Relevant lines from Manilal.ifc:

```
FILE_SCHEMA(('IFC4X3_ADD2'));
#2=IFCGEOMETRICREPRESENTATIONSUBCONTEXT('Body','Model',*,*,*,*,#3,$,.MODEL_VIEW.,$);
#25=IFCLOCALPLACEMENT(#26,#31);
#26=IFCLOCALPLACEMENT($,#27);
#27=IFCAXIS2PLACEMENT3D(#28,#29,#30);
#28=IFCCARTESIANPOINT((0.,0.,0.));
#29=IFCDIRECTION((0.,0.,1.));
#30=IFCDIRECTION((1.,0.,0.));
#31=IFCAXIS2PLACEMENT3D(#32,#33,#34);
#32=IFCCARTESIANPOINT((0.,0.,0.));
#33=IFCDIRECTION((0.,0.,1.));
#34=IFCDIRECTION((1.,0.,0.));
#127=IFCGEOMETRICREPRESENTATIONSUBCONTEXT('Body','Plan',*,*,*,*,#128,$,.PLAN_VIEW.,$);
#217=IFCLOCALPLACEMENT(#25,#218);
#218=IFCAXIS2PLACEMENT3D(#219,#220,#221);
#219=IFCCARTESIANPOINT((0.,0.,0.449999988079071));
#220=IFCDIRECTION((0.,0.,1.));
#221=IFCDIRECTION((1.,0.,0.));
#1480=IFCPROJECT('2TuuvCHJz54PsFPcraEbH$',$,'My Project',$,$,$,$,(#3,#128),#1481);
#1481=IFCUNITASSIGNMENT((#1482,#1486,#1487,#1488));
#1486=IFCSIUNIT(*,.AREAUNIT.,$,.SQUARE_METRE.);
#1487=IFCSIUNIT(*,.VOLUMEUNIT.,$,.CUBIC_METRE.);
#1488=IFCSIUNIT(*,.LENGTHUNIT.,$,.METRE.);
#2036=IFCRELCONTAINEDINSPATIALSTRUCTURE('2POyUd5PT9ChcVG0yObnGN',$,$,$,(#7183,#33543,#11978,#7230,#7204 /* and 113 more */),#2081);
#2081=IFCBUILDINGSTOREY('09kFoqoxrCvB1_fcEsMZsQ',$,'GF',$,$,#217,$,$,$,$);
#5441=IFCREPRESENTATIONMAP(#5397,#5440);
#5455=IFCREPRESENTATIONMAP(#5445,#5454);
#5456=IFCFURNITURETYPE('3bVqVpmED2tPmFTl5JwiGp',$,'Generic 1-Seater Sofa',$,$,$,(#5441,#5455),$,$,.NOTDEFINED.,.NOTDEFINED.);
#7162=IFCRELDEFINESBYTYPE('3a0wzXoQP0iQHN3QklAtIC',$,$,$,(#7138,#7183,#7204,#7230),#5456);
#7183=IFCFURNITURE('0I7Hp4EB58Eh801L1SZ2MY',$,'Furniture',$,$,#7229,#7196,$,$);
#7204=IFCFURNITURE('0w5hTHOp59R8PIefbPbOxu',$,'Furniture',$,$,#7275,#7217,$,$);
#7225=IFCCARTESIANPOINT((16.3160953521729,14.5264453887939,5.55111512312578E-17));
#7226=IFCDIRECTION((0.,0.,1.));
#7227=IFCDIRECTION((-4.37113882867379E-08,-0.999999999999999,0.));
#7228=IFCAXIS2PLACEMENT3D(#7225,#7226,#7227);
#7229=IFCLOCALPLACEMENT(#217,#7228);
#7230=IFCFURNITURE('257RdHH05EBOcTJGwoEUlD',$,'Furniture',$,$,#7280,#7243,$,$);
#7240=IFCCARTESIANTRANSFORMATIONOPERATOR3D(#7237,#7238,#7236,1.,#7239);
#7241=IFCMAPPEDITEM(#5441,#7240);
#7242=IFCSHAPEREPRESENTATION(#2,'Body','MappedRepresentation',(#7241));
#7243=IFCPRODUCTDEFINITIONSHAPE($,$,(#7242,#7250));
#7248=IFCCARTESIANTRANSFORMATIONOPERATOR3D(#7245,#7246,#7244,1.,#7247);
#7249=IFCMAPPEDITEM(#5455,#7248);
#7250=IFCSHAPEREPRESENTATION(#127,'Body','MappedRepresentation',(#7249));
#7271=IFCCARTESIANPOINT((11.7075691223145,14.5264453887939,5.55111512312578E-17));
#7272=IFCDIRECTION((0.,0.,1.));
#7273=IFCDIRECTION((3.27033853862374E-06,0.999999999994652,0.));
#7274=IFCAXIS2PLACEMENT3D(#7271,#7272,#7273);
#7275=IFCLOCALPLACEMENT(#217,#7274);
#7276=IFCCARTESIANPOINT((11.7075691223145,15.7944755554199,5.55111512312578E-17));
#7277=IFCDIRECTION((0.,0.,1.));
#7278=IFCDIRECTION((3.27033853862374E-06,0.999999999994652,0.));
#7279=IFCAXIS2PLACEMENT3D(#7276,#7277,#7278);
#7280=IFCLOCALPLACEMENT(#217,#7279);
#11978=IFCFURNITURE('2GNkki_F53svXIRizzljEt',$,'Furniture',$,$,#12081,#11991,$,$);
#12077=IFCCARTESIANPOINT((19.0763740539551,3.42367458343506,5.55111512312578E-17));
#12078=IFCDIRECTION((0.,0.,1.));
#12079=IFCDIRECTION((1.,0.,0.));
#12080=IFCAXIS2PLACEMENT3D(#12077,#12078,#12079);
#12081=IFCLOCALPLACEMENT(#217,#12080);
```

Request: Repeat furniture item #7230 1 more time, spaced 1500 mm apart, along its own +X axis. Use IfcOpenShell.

```python
import ifcopenshell
import ifcopenshell.api.geometry
import ifcopenshell.api.root
import ifcopenshell.util.element
import ifcopenshell.util.placement

model = ifcopenshell.open("Manilal.ifc")

source = model.by_id(7230)
base = ifcopenshell.util.placement.get_local_placement(source.ObjectPlacement)
step = base[:3, 0] * 1.5

for i in range(1, 2):
    copy = ifcopenshell.api.root.copy_class(model, product=source)
    copy.Representation = ifcopenshell.util.element.copy_deep(
        model, source.Representation, exclude=["IfcGeometricRepresentationContext", "IfcRepresentationMap"]
    )
    matrix = base.copy()
    matrix[:3, 3] += i * step
    print("added at", matrix[:3, 3].round(3) + 0.0)
    ifcopenshell.api.geometry.edit_object_placement(model, product=copy, matrix=matrix, is_si=False)

model.write("Manilal_updated.ifc")
```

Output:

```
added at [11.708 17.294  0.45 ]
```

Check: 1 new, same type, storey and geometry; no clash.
